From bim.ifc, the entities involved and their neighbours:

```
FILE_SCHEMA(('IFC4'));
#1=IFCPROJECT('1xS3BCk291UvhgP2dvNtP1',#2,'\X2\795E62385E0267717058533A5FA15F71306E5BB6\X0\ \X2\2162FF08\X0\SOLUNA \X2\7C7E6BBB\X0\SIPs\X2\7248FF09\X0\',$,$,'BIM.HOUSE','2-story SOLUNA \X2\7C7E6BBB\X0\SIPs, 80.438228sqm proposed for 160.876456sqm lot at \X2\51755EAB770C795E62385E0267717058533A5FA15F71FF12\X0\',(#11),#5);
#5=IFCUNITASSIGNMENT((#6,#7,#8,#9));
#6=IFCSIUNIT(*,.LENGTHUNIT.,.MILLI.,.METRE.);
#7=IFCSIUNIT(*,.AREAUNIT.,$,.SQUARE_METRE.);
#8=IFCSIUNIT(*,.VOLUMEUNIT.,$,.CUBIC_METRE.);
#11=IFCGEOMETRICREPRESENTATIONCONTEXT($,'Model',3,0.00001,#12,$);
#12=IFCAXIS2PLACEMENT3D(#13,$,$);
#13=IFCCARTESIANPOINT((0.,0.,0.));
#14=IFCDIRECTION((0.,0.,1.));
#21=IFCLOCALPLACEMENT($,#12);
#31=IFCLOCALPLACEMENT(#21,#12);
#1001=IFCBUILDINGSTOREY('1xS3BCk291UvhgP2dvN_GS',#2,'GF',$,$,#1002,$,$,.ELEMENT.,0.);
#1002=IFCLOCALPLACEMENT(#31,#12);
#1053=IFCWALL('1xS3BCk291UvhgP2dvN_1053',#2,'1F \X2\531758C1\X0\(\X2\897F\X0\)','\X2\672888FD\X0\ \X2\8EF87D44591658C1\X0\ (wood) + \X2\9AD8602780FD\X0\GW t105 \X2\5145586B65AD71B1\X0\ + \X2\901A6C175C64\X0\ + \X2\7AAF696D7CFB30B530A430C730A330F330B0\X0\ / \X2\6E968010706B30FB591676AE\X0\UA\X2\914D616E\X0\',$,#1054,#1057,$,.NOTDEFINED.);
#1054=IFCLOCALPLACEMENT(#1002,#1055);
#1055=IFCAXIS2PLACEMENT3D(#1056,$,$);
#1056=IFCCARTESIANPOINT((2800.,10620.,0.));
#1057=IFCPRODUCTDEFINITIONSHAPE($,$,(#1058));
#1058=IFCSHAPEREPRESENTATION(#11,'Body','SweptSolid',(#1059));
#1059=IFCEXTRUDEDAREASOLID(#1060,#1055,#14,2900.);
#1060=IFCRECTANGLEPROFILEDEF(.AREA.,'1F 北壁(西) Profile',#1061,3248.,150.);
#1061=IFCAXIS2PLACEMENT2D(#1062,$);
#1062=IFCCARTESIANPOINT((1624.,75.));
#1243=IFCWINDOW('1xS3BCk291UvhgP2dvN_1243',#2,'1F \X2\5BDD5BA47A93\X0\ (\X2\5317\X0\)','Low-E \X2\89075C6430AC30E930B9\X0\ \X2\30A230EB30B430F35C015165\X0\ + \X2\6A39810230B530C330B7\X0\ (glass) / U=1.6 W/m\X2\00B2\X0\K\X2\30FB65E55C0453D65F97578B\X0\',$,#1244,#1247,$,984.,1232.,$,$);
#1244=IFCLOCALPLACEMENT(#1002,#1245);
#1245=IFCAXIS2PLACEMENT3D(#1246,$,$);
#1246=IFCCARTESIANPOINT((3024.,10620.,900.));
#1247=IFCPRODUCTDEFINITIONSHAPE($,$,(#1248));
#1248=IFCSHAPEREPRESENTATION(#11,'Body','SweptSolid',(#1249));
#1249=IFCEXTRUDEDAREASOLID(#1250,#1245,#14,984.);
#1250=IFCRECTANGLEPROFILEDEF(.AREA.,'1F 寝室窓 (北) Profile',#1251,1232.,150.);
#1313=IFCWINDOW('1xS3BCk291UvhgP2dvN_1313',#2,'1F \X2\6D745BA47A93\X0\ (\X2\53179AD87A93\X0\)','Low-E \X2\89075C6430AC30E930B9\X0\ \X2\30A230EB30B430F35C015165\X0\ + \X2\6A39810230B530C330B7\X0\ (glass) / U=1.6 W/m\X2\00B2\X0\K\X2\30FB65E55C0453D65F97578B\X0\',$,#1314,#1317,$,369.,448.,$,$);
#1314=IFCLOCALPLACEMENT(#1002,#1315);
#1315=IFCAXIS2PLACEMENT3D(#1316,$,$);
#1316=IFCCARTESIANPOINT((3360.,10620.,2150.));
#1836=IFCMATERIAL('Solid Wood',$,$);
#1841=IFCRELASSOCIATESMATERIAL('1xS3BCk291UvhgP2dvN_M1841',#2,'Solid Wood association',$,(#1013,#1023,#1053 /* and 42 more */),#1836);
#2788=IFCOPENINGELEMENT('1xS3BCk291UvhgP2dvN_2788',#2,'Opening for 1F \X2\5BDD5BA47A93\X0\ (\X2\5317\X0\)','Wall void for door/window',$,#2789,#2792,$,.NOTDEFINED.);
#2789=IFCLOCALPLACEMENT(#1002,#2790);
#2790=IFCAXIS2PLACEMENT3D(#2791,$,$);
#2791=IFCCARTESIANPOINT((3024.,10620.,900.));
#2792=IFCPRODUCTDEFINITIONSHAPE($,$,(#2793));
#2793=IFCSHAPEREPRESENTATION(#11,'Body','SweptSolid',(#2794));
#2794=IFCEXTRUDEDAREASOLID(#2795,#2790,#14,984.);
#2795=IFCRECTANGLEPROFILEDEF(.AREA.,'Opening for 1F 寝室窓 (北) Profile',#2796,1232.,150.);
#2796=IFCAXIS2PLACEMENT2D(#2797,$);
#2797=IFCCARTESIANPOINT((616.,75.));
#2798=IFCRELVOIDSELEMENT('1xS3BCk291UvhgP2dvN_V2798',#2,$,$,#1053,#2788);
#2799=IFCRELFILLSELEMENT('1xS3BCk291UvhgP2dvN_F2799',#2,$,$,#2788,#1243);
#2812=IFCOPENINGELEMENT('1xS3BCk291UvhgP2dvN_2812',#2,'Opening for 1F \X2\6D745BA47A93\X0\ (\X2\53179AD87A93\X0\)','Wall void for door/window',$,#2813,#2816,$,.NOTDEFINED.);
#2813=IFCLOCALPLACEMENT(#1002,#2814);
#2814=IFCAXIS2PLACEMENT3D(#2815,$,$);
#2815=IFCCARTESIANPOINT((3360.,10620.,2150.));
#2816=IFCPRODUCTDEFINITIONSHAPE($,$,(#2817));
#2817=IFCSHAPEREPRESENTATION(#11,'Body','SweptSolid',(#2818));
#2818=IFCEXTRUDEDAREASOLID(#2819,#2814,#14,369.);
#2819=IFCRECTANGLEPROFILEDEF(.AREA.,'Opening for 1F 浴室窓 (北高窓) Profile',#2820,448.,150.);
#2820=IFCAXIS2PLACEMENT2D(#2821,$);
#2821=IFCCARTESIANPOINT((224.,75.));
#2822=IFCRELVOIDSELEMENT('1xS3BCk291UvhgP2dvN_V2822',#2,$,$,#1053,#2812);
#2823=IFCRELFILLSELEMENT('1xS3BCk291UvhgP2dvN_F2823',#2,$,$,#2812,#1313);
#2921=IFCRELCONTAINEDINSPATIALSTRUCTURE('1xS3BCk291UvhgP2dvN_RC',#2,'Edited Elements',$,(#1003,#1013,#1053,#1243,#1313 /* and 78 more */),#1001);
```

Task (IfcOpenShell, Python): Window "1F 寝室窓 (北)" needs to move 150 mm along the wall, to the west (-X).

```python
import ifcopenshell
import ifcopenshell.api.geometry
import ifcopenshell.util.placement
import ifcopenshell.util.unit

model = ifcopenshell.open("bim.ifc")
unit_scale = ifcopenshell.util.unit.calculate_unit_scale(model)

window = model.by_guid("1xS3BCk291UvhgP2dvN_1243")
opening = window.FillsVoids[0].RelatingOpeningElement
wall = opening.VoidsElements[0].RelatingBuildingElement

wall_matrix = ifcopenshell.util.placement.get_local_placement(wall.ObjectPlacement)
shift = wall_matrix[:3, 0] * -0.15 / unit_scale
before = ifcopenshell.util.placement.get_local_placement(window.ObjectPlacement)[:3, 3].copy()

# The window is not placed relative to its opening, so move both.
for product in (opening, window):
    matrix = ifcopenshell.util.placement.get_local_placement(product.ObjectPlacement)
    matrix[:3, 3] += shift
    ifcopenshell.api.geometry.edit_object_placement(model, product=product, matrix=matrix, is_si=False)

after = ifcopenshell.util.placement.get_local_placement(window.ObjectPlacement)[:3, 3]
print("window moved by", (after - before).round(3) + 0.0)

model.write("bim_v2.ifc")
```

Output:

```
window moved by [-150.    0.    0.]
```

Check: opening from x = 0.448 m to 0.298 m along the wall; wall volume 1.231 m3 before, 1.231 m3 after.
